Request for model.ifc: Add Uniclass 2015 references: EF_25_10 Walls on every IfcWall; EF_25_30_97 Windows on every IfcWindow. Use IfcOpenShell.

First a look at what the model holds.

```python
import ifcopenshell

model = ifcopenshell.open("model.ifc")
print(model.schema)
print("classifications:", [c.Name for c in model.by_type("IfcClassification")])
for ifc_class in ("IfcDoor", "IfcRoof", "IfcStair", "IfcWall", "IfcWindow"):
    print(ifc_class, len(model.by_type(ifc_class)))
```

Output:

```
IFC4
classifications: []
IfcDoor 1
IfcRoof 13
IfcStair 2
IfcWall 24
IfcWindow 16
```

```python
import ifcopenshell
import ifcopenshell.api.classification

model = ifcopenshell.open("model.ifc")

system = ifcopenshell.api.classification.add_classification(model, classification="Uniclass 2015")

codes = {
    "IfcWall": ("EF_25_10", "Walls"),
    "IfcWindow": ("EF_25_30_97", "Windows"),
}
for ifc_class, (code, name) in codes.items():
    products = model.by_type(ifc_class)
    ifcopenshell.api.classification.add_reference(
        model, products=products, classification=system, identification=code, name=name
    )
    print(code, len(products))

model.write("model_edited.ifc")
```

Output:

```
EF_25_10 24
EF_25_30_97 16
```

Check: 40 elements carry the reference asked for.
